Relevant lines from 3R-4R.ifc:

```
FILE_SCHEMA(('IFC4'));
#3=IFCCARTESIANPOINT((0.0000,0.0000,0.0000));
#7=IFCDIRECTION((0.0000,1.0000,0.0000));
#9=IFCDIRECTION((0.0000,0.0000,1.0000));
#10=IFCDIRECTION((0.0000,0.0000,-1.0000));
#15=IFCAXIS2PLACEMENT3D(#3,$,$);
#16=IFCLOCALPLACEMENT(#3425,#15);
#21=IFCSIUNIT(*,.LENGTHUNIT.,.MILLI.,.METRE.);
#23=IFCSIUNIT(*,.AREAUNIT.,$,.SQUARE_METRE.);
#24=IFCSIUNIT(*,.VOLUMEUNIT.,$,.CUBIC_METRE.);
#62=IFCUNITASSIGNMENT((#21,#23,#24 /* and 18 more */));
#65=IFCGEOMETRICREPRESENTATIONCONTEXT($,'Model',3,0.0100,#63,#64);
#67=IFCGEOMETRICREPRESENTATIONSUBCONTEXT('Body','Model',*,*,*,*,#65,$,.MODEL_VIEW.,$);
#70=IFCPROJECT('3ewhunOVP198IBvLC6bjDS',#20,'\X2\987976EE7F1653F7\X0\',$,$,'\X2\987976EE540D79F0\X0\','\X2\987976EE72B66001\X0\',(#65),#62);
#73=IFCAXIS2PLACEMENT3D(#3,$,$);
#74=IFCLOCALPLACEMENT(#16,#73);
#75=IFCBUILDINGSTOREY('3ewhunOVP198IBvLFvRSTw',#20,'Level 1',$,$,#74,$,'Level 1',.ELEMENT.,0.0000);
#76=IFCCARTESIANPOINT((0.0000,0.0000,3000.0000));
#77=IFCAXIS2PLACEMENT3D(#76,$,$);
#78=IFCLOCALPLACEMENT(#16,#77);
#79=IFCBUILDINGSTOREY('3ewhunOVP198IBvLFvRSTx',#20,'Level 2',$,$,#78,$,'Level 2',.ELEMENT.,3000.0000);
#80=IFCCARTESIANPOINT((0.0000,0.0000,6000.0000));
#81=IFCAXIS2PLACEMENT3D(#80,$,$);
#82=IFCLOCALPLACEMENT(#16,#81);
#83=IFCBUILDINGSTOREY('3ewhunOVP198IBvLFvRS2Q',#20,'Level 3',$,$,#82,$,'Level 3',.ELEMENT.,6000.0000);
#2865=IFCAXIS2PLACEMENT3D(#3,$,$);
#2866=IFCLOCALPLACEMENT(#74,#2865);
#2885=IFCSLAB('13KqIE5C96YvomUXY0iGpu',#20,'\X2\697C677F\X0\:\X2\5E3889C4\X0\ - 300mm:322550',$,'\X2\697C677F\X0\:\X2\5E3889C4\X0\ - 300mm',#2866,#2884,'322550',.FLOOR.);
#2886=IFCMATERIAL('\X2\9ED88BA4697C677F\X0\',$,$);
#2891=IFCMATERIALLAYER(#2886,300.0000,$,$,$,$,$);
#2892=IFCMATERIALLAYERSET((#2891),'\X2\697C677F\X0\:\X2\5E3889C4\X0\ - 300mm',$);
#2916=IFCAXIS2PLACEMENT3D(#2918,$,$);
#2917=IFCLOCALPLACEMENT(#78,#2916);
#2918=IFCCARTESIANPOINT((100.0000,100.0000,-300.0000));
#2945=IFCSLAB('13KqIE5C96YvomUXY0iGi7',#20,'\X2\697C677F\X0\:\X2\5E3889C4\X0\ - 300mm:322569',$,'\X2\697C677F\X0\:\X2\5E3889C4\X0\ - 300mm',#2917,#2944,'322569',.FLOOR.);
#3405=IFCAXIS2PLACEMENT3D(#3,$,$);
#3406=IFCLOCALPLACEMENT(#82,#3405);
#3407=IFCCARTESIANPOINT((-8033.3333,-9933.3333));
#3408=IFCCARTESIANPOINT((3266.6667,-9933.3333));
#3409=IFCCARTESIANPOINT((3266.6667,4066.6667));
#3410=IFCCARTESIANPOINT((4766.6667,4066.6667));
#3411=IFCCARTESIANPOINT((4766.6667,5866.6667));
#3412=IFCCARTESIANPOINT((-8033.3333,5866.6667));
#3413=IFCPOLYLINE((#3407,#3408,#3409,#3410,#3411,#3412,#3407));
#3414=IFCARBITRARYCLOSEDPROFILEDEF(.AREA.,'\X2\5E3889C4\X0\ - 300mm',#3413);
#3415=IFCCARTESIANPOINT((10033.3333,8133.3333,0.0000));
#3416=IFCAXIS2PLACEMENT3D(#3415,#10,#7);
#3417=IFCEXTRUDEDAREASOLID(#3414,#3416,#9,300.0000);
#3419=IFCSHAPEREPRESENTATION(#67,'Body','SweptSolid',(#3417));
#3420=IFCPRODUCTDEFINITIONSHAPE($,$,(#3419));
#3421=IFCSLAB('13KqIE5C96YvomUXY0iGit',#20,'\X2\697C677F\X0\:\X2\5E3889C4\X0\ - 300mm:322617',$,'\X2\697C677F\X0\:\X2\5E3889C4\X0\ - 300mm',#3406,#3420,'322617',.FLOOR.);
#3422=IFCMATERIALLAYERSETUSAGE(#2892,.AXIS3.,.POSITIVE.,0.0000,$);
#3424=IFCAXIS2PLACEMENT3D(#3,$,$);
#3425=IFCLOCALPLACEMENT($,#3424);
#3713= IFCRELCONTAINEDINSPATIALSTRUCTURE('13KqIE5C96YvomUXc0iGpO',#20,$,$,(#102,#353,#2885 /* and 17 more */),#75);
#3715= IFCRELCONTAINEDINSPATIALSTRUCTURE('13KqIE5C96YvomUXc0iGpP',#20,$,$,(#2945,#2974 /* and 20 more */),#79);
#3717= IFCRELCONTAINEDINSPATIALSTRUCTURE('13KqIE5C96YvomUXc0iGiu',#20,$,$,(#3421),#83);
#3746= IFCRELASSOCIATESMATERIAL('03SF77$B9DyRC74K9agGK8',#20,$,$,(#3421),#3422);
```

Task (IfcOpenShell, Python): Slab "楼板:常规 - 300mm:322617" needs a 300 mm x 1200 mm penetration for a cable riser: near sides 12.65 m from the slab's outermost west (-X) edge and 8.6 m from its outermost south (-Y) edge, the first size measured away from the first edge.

```python
import numpy as np
import ifcopenshell
import ifcopenshell.api.feature
import ifcopenshell.api.geometry
import ifcopenshell.api.root
import ifcopenshell.geom
import ifcopenshell.util.placement
import ifcopenshell.util.representation
import ifcopenshell.util.shape
import ifcopenshell.util.unit

model = ifcopenshell.open("3R-4R.ifc")
unit_scale = ifcopenshell.util.unit.calculate_unit_scale(model)
settings = ifcopenshell.geom.settings()


def volume(element):
    """Net volume in cubic metres, openings subtracted."""
    shape = ifcopenshell.geom.create_shape(settings, element)
    return ifcopenshell.util.shape.get_volume(shape.geometry)


slab = model.by_guid("13KqIE5C96YvomUXY0iGit")
before = volume(slab)

# Extent in the slab's own axes, in metres. The edges named are its -X and -Y sides.
slab_shape = ifcopenshell.geom.create_shape(settings, slab)
vertices = ifcopenshell.util.shape.get_vertices(slab_shape.geometry)
x_min, y_min, bottom = vertices.min(axis=0)
top = vertices[:, 2].max()

opening = ifcopenshell.api.root.create_entity(model, ifc_class="IfcOpeningElement", name="Cable riser opening", predefined_type="OPENING")
context = ifcopenshell.util.representation.get_context(model, "Model", "Body", "MODEL_VIEW")
width, depth = 0.3, 1.2
outline = [(0.0, 0.0), (width, 0.0), (width, depth), (0.0, depth), (0.0, 0.0)]
# Overshoot both faces by 50 mm so the cut is clean.
shape = ifcopenshell.api.geometry.add_slab_representation(
    model, context=context, depth=top - bottom + 0.1, polyline=outline
)
ifcopenshell.api.geometry.assign_representation(model, product=opening, representation=shape)

matrix = ifcopenshell.util.placement.get_local_placement(slab.ObjectPlacement)
matrix[:, 3] = matrix @ np.append(np.array([x_min + 12.65, y_min + 8.6, bottom - 0.05]) / unit_scale, 1.0)
ifcopenshell.api.geometry.edit_object_placement(model, product=opening, matrix=matrix, is_si=False)
ifcopenshell.api.feature.add_feature(model, feature=opening, element=slab)

after = volume(slab)

print(f"slab volume {before:.3f} -> {after:.3f} m3")

model.write("3R-4R_rev.ifc")
```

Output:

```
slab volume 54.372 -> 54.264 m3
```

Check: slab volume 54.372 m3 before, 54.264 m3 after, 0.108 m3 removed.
